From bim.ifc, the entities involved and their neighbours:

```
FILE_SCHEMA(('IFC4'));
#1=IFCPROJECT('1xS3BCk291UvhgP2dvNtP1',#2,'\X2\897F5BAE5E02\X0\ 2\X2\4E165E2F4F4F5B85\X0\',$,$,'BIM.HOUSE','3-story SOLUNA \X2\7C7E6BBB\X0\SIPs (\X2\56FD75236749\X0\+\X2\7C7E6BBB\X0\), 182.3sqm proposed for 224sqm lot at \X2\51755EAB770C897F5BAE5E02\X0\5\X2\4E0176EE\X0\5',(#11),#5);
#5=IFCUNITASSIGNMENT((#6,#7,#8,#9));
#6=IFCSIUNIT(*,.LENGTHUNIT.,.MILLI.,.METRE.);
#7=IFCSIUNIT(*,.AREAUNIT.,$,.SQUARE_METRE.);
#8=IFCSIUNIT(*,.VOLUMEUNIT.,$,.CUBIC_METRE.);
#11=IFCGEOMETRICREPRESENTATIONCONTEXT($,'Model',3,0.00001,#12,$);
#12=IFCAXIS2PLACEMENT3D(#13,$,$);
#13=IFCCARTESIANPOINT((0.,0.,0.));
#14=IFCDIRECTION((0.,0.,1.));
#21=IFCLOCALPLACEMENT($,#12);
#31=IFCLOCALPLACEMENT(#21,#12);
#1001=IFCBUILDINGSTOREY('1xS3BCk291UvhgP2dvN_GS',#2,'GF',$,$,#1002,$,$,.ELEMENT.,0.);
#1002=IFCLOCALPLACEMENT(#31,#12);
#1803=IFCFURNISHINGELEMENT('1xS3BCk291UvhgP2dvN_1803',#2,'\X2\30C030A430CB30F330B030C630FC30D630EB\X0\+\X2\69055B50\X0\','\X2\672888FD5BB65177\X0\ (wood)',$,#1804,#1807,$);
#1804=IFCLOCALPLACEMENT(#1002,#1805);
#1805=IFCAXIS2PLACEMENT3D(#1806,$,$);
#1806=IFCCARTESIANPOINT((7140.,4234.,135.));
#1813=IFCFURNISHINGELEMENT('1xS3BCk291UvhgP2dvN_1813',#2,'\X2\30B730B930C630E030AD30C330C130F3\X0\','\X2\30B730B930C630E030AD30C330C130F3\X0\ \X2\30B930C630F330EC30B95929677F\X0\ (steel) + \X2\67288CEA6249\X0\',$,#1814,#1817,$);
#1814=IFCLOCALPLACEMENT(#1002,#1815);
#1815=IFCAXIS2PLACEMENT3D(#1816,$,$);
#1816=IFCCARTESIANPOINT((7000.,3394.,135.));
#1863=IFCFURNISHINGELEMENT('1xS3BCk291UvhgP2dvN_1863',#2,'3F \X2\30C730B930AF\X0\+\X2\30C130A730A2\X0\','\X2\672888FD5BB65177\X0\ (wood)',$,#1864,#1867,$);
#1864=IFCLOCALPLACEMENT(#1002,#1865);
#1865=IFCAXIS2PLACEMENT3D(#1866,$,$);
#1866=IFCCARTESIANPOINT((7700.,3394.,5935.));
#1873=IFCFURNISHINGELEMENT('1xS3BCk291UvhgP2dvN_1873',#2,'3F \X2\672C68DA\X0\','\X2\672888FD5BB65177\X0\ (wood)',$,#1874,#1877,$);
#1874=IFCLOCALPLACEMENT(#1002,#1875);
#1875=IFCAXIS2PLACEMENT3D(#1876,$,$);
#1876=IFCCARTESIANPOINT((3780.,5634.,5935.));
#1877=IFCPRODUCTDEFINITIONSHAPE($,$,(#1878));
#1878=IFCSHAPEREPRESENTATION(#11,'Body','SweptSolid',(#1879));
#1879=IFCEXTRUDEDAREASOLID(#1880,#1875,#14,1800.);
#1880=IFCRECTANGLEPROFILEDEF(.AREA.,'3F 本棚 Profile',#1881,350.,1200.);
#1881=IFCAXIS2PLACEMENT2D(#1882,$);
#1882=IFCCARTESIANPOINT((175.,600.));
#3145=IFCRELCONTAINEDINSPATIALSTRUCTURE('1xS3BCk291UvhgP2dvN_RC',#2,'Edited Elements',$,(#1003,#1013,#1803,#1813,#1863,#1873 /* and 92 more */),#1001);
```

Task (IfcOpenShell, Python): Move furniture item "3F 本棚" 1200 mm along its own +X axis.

```python
import ifcopenshell
import ifcopenshell.api.geometry
import ifcopenshell.util.placement
import ifcopenshell.util.unit

model = ifcopenshell.open("bim.ifc")
unit_scale = ifcopenshell.util.unit.calculate_unit_scale(model)

item = model.by_guid("1xS3BCk291UvhgP2dvN_1873")
matrix = ifcopenshell.util.placement.get_local_placement(item.ObjectPlacement)
matrix[:3, 3] += matrix[:3, 0] * 1.2 / unit_scale
ifcopenshell.api.geometry.edit_object_placement(model, product=item, matrix=matrix, is_si=False)

print(ifcopenshell.util.placement.get_local_placement(item.ObjectPlacement).round(3) + 0.0)

model.write("bim_edited.ifc")
```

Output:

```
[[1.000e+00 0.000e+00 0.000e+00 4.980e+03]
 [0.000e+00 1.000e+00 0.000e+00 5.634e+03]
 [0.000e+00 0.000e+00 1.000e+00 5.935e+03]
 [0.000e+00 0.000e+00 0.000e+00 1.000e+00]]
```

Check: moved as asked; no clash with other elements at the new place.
